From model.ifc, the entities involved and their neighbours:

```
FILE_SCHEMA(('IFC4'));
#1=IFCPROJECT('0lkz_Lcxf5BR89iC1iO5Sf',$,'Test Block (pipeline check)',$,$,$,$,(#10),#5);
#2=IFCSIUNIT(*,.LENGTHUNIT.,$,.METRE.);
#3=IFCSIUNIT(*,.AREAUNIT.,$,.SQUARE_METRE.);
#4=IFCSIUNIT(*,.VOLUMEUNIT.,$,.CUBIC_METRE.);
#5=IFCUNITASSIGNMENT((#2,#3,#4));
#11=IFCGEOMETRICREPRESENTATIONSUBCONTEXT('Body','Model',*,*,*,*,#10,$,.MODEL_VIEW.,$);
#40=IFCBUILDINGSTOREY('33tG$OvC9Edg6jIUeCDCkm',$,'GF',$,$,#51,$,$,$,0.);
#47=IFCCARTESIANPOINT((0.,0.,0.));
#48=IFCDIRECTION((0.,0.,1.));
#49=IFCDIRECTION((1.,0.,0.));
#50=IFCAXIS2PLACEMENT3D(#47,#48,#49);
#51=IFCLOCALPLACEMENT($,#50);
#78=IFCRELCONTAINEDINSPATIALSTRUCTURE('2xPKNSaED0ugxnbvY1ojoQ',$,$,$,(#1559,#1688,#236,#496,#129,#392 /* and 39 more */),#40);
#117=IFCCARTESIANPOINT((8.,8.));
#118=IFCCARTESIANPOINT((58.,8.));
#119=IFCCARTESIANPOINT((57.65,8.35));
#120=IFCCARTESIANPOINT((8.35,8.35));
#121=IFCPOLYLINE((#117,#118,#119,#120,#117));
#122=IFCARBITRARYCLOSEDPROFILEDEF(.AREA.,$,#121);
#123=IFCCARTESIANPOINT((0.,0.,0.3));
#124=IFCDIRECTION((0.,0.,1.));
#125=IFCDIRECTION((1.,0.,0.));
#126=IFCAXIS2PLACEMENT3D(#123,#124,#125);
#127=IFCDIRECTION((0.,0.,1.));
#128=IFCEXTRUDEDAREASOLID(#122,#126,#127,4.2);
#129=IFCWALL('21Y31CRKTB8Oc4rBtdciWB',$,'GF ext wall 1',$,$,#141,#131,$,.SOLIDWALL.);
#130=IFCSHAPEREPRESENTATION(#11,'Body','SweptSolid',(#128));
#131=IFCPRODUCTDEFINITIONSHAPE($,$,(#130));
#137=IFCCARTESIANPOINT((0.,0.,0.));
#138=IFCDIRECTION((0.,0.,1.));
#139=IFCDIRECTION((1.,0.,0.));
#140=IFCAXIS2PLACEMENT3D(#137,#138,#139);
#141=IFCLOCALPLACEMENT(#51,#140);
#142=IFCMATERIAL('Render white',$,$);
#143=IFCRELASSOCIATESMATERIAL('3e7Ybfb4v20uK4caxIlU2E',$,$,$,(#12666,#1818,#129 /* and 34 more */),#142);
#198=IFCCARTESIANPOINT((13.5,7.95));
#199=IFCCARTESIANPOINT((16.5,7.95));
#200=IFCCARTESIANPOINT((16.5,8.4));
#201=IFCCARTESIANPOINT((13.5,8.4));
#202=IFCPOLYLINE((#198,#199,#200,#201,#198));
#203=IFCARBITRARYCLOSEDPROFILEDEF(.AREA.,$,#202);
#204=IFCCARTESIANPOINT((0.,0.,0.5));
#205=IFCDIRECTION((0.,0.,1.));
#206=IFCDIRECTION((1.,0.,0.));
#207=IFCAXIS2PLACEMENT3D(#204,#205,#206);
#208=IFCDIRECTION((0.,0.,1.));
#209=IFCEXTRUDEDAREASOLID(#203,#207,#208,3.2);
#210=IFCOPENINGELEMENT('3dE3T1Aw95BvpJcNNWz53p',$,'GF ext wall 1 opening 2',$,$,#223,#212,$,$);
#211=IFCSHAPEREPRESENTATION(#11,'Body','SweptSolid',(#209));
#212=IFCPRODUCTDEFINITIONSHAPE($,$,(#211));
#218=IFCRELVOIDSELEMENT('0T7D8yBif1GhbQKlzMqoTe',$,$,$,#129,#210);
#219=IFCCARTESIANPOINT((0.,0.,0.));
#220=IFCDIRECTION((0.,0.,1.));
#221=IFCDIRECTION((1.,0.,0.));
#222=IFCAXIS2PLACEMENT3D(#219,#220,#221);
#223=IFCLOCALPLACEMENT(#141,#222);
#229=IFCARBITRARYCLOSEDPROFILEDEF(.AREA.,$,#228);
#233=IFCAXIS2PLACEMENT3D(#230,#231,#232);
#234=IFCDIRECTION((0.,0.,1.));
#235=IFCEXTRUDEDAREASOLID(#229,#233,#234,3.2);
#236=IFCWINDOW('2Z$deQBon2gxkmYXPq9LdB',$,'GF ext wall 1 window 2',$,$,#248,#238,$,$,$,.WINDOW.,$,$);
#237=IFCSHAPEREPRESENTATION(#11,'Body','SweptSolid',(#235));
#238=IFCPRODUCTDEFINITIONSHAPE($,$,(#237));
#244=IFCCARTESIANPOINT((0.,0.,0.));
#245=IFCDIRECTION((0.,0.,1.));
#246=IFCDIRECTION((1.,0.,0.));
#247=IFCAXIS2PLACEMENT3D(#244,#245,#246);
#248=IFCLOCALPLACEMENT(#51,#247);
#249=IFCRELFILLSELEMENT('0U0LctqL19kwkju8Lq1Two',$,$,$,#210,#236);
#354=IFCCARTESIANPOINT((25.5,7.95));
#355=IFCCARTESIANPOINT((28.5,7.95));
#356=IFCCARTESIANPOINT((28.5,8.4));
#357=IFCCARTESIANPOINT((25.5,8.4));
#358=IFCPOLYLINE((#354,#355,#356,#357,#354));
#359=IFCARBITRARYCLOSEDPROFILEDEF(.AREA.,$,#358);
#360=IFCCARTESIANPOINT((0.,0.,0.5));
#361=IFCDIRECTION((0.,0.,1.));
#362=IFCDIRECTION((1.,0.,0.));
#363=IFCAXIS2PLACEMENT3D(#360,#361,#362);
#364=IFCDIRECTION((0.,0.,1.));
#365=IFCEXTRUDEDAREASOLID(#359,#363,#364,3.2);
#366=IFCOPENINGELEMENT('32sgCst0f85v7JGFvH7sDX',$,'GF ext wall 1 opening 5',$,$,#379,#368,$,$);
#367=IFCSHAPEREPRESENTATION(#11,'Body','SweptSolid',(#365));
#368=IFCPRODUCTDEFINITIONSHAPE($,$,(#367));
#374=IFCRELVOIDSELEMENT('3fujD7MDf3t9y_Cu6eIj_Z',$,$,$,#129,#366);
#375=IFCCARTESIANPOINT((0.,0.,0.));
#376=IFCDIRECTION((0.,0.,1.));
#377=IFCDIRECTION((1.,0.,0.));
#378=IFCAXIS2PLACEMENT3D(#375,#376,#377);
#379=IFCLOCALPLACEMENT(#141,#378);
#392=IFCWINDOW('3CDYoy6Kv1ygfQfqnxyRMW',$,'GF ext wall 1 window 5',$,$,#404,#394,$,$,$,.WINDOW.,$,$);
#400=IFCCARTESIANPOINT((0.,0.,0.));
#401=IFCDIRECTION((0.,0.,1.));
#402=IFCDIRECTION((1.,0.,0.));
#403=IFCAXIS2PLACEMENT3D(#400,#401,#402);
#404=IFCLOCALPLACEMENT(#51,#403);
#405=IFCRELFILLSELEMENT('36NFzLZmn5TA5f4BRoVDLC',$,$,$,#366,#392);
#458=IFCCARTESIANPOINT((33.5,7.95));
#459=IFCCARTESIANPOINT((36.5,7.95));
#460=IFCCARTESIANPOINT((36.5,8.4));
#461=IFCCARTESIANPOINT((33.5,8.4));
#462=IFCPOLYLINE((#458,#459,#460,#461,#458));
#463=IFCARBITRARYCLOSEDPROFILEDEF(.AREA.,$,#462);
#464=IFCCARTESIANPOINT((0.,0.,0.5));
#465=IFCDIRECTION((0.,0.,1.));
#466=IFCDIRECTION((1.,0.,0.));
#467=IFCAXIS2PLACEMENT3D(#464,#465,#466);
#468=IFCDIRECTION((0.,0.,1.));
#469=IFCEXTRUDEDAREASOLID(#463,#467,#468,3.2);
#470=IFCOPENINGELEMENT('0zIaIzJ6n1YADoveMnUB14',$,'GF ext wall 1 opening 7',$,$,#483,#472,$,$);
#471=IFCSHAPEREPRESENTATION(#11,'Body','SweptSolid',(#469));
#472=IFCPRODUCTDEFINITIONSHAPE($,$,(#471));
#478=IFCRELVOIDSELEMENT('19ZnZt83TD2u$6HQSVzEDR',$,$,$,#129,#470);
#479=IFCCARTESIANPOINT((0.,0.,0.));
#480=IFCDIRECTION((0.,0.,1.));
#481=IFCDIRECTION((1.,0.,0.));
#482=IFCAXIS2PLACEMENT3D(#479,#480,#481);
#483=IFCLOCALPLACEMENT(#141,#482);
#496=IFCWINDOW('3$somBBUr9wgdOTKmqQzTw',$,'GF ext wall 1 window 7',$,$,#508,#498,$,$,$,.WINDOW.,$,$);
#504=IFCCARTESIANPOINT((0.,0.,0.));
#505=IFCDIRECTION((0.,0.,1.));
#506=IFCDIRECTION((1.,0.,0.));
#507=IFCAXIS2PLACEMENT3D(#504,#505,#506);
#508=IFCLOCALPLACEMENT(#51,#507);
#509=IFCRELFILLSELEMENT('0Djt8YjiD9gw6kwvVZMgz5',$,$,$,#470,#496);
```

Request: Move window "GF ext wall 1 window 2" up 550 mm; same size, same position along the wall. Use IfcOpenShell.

```python
import numpy as np
import ifcopenshell
import ifcopenshell.api.geometry
import ifcopenshell.util.placement
import ifcopenshell.util.unit

model = ifcopenshell.open("model.ifc")
unit_scale = ifcopenshell.util.unit.calculate_unit_scale(model)

window = model.by_guid("2Z$deQBon2gxkmYXPq9LdB")
opening = window.FillsVoids[0].RelatingOpeningElement
dz = 0.55

shift = np.array([0.0, 0.0, dz])
# The window is not placed relative to its opening, so move both.
for product in (opening, window):
    matrix = ifcopenshell.util.placement.get_local_placement(product.ObjectPlacement)
    matrix[:3, 3] += shift
    ifcopenshell.api.geometry.edit_object_placement(model, product=product, matrix=matrix, is_si=False)

print(f"moved by {dz * unit_scale:+.3f} m")

model.write("model_updated.ifc")
```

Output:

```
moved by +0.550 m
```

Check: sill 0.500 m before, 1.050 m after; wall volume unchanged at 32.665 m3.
